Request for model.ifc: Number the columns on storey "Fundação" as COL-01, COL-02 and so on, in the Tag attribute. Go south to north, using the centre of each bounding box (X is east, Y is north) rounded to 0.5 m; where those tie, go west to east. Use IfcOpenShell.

First a look at what the model holds.

```python
import ifcopenshell
import ifcopenshell.util.element
import ifcopenshell.util.placement

model = ifcopenshell.open("model.ifc")
print(model.schema)
storey = next(s for s in model.by_type("IfcBuildingStorey") if s.Name == "Fundação")
columns = [e for e in ifcopenshell.util.element.get_decomposition(storey) if e.is_a("IfcColumn")]
for e in sorted(columns, key=lambda e: e.id()):
    origin = ifcopenshell.util.placement.get_local_placement(e.ObjectPlacement)[:3, 3]
    print(e.id(), e.Tag, e.Name, origin.round(2) + 0.0, sep=" | ")
```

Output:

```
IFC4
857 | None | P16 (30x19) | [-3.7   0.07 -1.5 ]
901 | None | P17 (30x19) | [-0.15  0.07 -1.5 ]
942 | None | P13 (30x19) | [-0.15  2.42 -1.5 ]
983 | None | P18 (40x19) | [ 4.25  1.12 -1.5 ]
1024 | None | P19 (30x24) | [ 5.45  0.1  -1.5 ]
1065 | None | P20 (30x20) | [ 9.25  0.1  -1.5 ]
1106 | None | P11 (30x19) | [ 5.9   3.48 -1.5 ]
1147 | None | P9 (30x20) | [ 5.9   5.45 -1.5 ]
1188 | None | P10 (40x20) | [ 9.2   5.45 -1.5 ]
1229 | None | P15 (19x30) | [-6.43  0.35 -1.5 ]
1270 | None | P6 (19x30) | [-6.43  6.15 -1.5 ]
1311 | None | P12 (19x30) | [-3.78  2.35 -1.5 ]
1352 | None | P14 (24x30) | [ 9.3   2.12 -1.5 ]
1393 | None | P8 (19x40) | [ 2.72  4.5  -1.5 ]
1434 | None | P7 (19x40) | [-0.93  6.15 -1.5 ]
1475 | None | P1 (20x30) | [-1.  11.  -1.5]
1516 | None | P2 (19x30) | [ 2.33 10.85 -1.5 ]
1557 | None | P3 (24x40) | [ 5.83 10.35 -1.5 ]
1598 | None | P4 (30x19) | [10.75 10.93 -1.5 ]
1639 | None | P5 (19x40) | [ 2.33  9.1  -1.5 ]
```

```python
import ifcopenshell
import ifcopenshell.geom
import ifcopenshell.util.element
import ifcopenshell.util.shape

model = ifcopenshell.open("model.ifc")
settings = ifcopenshell.geom.settings()
settings.set("use-world-coords", True)


def centre(element):
    shape = ifcopenshell.geom.create_shape(settings, element)
    return ifcopenshell.util.shape.get_bbox_centroid(shape.geometry)


storey = next(s for s in model.by_type("IfcBuildingStorey") if s.Name == "Fundação")
columns = [e for e in ifcopenshell.util.element.get_decomposition(storey) if e.is_a("IfcColumn")]

# Insertion points can sit at a corner or the storey origin, so sort by the geometry (in metres).
centres = {e: centre(e) for e in columns}
columns.sort(key=lambda e: (round(centres[e][1] / 0.5), centres[e][0]))

for i, e in enumerate(columns, start=1):
    number = f"COL-{i:02d}"
    e.Tag = number
    print(e.id(), number)

model.write("model_edited.ifc")
```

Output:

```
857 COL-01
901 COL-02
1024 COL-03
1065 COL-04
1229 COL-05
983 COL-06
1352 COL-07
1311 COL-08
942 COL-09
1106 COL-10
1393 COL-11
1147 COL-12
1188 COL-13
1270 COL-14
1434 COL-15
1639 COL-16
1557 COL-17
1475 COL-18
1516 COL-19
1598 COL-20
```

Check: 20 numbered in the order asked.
